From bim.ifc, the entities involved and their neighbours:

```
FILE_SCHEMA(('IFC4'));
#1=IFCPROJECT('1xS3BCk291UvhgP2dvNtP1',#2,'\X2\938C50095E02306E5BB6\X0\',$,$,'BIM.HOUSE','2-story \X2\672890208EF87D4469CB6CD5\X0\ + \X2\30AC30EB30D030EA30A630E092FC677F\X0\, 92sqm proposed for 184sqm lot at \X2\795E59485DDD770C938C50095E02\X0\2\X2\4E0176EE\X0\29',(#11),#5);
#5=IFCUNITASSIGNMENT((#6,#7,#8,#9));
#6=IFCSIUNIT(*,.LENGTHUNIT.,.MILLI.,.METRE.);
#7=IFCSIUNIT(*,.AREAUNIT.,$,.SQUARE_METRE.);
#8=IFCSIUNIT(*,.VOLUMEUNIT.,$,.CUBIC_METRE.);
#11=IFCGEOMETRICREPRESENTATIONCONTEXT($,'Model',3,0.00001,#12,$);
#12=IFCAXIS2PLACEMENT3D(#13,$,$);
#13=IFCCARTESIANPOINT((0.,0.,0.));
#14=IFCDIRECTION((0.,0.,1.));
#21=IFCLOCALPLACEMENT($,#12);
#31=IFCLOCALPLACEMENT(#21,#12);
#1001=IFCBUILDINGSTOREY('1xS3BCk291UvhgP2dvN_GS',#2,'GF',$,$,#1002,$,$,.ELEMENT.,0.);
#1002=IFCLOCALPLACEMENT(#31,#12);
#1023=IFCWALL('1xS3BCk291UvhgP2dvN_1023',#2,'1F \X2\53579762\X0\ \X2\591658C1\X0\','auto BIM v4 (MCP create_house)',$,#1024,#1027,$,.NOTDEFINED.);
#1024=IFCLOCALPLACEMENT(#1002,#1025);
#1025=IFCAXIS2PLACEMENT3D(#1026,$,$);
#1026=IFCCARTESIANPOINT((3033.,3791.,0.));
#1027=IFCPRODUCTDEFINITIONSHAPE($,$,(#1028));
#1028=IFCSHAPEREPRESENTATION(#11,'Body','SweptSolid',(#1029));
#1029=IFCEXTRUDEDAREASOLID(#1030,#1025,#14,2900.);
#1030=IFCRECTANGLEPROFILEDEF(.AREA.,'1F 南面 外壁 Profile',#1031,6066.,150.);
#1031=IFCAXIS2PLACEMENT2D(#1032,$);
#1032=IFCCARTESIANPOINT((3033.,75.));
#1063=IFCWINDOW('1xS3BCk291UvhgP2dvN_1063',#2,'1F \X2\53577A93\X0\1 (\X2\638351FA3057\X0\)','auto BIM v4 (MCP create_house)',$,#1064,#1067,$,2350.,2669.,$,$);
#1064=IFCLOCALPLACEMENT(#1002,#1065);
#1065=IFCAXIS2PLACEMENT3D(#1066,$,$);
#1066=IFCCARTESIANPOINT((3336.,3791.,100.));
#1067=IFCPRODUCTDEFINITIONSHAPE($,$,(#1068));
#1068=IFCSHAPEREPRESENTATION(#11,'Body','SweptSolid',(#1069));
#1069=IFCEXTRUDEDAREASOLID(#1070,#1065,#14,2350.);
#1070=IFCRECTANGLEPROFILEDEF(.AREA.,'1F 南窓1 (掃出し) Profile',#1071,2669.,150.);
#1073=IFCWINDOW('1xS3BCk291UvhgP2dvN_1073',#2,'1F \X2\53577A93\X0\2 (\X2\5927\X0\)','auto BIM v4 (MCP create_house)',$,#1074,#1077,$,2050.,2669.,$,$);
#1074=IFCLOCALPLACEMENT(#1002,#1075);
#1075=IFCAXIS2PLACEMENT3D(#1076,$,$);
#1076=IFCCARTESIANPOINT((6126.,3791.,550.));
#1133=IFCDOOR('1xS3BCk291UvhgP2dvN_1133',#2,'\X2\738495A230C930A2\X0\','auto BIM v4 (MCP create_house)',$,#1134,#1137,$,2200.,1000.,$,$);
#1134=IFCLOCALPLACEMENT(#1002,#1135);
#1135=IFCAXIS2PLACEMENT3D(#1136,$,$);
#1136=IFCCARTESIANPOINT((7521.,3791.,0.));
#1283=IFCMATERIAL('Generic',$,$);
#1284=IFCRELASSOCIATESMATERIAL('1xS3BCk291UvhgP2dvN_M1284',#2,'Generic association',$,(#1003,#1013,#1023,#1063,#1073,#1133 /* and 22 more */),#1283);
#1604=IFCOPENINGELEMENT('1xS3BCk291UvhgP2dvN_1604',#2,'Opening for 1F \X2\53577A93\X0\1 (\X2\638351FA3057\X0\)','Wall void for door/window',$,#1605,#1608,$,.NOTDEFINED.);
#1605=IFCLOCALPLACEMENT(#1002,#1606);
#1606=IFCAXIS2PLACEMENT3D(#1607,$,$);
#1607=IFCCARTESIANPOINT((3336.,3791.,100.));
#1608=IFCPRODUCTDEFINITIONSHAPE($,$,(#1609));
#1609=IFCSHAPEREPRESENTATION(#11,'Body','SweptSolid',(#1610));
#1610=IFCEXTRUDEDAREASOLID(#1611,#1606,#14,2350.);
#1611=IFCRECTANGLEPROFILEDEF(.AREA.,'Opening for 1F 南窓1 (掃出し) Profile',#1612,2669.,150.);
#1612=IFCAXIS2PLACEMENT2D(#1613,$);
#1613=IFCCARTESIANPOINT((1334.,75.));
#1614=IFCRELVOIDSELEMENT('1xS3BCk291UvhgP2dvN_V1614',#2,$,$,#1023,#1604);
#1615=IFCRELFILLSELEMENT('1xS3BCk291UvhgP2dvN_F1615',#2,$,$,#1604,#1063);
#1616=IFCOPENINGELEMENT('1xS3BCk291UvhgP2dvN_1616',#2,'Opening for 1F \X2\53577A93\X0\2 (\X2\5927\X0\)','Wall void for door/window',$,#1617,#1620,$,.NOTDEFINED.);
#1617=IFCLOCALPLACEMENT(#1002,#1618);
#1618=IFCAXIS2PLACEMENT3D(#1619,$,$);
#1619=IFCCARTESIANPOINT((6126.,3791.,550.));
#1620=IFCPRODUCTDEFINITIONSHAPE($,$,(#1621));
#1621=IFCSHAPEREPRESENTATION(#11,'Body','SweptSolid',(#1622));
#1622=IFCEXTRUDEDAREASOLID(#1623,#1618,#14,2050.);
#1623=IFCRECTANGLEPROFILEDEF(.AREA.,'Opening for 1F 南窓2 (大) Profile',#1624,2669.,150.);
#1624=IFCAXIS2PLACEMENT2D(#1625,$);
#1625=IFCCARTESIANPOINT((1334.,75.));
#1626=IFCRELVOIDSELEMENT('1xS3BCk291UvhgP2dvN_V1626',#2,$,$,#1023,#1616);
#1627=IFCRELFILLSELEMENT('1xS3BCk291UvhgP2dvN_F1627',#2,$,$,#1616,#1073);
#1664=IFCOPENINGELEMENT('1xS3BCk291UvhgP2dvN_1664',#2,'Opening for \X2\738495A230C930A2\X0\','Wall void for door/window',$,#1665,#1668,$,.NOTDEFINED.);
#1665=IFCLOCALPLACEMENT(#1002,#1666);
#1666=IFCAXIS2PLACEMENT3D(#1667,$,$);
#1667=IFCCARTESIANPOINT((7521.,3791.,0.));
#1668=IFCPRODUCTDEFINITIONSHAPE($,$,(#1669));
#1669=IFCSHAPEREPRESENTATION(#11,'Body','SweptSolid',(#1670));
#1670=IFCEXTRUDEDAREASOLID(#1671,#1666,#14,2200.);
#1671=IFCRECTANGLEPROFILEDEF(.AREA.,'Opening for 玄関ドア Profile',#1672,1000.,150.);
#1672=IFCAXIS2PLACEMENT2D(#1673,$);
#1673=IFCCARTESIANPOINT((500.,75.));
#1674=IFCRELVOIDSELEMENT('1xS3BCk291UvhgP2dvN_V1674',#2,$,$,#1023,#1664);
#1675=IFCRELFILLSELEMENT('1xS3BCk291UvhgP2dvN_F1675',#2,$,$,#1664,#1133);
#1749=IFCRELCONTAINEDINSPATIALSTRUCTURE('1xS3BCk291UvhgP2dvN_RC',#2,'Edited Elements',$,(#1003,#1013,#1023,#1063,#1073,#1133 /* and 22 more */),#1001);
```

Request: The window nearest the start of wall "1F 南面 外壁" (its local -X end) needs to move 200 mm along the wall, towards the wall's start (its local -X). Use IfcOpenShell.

```python
import ifcopenshell
import ifcopenshell.api.geometry
import ifcopenshell.util.placement
import ifcopenshell.util.unit

model = ifcopenshell.open("bim.ifc")
unit_scale = ifcopenshell.util.unit.calculate_unit_scale(model)

window = model.by_guid("1xS3BCk291UvhgP2dvN_1063")
opening = window.FillsVoids[0].RelatingOpeningElement
wall = opening.VoidsElements[0].RelatingBuildingElement

wall_matrix = ifcopenshell.util.placement.get_local_placement(wall.ObjectPlacement)
shift = wall_matrix[:3, 0] * -0.2 / unit_scale
before = ifcopenshell.util.placement.get_local_placement(window.ObjectPlacement)[:3, 3].copy()

# The window is not placed relative to its opening, so move both.
for product in (opening, window):
    matrix = ifcopenshell.util.placement.get_local_placement(product.ObjectPlacement)
    matrix[:3, 3] += shift
    ifcopenshell.api.geometry.edit_object_placement(model, product=product, matrix=matrix, is_si=False)

after = ifcopenshell.util.placement.get_local_placement(window.ObjectPlacement)[:3, 3]
print("window moved by", (after - before).round(3) + 0.0)

model.write("bim-out.ifc")
```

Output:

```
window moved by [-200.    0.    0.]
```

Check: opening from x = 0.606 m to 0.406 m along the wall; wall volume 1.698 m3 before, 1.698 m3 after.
